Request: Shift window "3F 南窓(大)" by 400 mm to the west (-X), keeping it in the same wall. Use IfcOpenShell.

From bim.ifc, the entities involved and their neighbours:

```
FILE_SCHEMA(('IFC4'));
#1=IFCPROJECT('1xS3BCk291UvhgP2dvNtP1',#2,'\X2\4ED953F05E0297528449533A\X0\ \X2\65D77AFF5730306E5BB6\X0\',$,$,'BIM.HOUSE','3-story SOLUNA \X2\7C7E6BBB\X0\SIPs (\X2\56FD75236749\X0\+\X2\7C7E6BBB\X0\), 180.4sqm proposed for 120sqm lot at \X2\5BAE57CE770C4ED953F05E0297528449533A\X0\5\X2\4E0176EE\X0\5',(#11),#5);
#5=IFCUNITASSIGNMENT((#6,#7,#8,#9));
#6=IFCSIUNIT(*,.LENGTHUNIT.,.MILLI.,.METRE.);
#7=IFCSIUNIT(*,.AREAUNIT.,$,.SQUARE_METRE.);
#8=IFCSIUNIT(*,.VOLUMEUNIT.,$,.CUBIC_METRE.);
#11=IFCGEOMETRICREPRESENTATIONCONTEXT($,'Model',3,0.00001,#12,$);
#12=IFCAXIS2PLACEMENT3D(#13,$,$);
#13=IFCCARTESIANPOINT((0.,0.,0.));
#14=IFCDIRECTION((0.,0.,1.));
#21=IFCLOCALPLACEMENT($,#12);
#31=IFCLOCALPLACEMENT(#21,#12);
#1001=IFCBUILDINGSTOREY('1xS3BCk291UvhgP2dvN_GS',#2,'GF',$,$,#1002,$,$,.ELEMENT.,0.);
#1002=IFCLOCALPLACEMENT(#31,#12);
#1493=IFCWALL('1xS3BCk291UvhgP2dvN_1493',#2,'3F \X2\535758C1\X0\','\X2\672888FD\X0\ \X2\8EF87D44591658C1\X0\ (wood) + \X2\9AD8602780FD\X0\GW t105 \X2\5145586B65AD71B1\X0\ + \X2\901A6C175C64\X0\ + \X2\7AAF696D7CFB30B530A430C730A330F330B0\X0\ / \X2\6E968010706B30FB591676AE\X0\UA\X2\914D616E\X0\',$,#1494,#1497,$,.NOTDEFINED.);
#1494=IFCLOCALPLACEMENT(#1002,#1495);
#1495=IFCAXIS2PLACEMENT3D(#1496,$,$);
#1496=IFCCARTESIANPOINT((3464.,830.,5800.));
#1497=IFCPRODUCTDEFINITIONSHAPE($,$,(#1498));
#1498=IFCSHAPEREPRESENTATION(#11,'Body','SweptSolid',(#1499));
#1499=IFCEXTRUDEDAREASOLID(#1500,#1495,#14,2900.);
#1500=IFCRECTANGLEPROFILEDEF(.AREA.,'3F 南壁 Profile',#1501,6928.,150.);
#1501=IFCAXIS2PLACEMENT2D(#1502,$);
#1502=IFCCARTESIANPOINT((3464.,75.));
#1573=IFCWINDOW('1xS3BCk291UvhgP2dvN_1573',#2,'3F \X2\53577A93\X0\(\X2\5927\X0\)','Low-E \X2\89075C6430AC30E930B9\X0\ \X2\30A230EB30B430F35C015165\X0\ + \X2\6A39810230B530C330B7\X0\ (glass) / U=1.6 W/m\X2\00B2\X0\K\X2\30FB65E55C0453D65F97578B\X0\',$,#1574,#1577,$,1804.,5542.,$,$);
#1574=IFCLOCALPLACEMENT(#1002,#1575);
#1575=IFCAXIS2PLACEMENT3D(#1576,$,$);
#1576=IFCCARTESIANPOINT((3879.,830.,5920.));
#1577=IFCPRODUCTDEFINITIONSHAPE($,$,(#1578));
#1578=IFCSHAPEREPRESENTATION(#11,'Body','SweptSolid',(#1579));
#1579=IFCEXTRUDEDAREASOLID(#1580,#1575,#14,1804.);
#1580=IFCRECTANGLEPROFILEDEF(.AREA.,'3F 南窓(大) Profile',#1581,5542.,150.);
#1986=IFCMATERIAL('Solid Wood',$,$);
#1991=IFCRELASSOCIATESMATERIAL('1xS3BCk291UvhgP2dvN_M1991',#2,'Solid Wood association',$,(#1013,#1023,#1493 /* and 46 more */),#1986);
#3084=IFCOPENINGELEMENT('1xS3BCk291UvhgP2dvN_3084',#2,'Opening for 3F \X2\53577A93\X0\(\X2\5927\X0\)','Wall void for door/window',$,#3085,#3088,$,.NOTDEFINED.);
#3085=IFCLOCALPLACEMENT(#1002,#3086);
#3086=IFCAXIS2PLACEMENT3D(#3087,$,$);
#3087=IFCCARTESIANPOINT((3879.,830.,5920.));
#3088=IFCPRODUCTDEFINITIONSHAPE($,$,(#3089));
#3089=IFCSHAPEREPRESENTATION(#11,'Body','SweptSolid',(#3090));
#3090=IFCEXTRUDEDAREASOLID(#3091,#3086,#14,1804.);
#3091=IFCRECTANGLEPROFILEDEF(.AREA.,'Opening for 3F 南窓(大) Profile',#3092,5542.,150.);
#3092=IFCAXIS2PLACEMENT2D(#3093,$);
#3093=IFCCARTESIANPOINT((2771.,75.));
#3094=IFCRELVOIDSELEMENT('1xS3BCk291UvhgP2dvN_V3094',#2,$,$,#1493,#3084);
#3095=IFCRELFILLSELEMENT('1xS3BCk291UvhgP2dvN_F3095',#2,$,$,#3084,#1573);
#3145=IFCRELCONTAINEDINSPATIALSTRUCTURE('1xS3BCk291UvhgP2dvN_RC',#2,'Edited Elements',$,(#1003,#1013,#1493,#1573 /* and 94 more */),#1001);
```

```python
import ifcopenshell
import ifcopenshell.api.geometry
import ifcopenshell.util.placement

model = ifcopenshell.open("bim.ifc")

window = model.by_guid("1xS3BCk291UvhgP2dvN_1573")
opening = window.FillsVoids[0].RelatingOpeningElement
wall = opening.VoidsElements[0].RelatingBuildingElement

wall_matrix = ifcopenshell.util.placement.get_local_placement(wall.ObjectPlacement)
shift = wall_matrix[:3, 0] * -400.0
before = ifcopenshell.util.placement.get_local_placement(window.ObjectPlacement)[:3, 3].copy()

# The window is not placed relative to its opening, so move both.
for product in (opening, window):
    matrix = ifcopenshell.util.placement.get_local_placement(product.ObjectPlacement)
    matrix[:3, 3] += shift
    ifcopenshell.api.geometry.edit_object_placement(model, product=product, matrix=matrix, is_si=False)

after = ifcopenshell.util.placement.get_local_placement(window.ObjectPlacement)[:3, 3]
print("window moved by", (after - before).round(3) + 0.0)

model.write("bim_updated.ifc")
```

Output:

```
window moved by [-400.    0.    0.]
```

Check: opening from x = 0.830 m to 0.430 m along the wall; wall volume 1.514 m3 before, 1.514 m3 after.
